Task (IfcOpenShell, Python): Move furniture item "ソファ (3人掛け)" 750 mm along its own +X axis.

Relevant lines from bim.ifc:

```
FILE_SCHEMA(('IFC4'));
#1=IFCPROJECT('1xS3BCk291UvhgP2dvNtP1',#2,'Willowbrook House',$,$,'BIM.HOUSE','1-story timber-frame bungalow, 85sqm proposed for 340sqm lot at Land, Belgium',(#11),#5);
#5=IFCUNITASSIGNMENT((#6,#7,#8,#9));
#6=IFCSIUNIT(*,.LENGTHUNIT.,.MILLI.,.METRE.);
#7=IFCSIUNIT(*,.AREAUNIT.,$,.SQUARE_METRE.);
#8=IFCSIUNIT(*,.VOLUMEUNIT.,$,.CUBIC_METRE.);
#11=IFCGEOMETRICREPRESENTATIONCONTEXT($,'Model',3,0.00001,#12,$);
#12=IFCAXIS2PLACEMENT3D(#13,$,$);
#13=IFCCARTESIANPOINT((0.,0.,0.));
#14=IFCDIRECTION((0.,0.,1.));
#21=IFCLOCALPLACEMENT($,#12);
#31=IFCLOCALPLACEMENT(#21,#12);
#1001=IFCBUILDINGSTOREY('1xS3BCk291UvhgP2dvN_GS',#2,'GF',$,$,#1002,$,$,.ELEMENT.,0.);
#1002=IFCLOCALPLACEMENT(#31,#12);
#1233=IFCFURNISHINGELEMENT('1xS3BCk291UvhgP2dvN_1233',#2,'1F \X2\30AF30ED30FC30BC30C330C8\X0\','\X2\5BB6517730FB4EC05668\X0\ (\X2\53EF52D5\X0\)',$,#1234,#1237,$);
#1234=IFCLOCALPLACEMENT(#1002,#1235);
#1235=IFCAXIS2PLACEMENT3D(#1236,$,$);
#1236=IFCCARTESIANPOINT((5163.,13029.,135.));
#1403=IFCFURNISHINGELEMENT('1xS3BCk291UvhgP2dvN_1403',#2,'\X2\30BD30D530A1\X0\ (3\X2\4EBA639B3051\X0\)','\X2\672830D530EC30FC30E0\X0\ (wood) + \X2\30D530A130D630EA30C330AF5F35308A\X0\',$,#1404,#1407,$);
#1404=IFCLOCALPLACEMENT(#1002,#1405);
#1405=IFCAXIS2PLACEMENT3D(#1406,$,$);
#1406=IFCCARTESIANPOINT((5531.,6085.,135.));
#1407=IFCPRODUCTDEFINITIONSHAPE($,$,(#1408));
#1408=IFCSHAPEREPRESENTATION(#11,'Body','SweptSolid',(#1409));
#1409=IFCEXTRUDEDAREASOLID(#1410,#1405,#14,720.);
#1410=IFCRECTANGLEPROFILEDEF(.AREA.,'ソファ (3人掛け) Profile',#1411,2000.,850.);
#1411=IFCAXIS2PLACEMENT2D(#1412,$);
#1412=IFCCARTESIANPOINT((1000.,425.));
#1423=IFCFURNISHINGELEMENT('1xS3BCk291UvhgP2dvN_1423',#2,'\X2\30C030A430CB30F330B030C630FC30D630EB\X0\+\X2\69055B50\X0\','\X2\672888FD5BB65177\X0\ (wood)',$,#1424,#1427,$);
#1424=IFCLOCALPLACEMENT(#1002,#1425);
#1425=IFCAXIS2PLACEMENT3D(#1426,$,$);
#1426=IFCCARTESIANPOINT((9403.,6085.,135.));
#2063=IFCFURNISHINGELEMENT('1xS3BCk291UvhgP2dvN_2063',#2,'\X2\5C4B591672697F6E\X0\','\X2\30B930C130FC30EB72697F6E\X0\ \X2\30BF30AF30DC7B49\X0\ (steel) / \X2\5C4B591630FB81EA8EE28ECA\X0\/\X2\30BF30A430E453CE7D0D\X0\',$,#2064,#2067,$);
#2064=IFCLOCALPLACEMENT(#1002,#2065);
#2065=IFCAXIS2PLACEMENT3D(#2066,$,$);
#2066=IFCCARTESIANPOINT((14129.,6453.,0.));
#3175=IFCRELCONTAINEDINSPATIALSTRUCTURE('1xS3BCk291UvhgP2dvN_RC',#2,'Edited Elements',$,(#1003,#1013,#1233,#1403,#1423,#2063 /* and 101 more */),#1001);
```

```python
import ifcopenshell
import ifcopenshell.api.geometry
import ifcopenshell.util.placement

model = ifcopenshell.open("bim.ifc")

item = model.by_guid("1xS3BCk291UvhgP2dvN_1403")
matrix = ifcopenshell.util.placement.get_local_placement(item.ObjectPlacement)
matrix[:3, 3] += matrix[:3, 0] * 750.0
ifcopenshell.api.geometry.edit_object_placement(model, product=item, matrix=matrix, is_si=False)

print(ifcopenshell.util.placement.get_local_placement(item.ObjectPlacement).round(3) + 0.0)

model.write("bim_updated.ifc")
```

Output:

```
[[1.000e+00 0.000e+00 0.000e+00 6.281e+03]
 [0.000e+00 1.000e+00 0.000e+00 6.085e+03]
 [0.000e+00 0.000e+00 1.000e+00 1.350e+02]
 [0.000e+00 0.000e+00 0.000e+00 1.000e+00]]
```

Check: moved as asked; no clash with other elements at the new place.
